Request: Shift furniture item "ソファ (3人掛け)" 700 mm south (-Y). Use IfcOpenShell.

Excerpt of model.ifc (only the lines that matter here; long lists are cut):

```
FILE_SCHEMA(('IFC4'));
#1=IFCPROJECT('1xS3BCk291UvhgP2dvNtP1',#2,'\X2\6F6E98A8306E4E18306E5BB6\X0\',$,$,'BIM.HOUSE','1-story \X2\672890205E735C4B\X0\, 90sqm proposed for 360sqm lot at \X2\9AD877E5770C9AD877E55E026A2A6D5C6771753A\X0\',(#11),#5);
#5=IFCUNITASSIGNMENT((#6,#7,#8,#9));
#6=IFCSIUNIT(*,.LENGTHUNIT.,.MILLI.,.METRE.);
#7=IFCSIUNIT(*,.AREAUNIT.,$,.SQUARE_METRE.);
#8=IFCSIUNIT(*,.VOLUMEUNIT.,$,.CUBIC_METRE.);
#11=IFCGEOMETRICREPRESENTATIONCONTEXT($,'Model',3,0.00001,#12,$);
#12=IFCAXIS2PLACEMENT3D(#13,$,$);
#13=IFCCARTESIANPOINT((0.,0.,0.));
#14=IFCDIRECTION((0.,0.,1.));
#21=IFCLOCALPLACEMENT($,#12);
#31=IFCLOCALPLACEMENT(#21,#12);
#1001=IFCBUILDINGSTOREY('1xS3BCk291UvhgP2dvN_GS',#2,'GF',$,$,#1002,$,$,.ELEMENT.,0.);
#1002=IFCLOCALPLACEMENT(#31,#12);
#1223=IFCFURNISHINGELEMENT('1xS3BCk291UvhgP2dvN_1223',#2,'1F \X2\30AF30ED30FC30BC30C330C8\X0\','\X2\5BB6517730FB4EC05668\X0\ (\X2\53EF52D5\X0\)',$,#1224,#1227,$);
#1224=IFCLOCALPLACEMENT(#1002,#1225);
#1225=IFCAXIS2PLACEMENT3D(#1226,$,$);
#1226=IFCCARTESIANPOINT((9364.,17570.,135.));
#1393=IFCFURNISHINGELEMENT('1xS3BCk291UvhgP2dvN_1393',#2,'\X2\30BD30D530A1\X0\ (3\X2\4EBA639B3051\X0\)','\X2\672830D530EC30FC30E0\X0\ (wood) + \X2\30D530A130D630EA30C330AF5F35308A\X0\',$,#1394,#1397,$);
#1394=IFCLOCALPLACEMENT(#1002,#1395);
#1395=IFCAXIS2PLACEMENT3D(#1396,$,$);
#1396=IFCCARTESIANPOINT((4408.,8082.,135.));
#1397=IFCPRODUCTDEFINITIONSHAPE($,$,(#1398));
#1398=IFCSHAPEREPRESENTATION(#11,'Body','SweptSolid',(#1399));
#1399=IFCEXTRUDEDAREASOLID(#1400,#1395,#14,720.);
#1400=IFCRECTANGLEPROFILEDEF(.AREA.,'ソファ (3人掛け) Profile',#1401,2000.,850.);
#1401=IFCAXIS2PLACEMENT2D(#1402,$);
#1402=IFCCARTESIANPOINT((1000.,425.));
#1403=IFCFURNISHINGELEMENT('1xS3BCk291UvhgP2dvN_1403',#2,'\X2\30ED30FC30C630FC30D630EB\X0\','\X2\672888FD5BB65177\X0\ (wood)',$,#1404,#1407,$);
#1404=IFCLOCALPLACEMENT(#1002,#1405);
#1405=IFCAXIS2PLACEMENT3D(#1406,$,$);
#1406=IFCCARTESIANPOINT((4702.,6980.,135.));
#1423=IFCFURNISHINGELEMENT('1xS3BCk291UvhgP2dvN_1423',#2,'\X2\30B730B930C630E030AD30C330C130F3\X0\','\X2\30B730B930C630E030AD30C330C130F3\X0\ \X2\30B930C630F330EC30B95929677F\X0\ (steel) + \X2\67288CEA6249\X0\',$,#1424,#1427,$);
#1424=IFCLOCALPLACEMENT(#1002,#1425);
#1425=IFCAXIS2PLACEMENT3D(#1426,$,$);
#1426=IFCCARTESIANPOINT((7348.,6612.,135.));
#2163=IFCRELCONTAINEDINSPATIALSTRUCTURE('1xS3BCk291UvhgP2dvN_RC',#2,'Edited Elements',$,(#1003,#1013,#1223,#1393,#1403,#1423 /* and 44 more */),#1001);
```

```python
import ifcopenshell
import ifcopenshell.api.geometry
import ifcopenshell.util.placement
import ifcopenshell.util.unit

model = ifcopenshell.open("model.ifc")
unit_scale = ifcopenshell.util.unit.calculate_unit_scale(model)

item = model.by_guid("1xS3BCk291UvhgP2dvN_1393")
matrix = ifcopenshell.util.placement.get_local_placement(item.ObjectPlacement)
matrix[1, 3] -= 0.7 / unit_scale
ifcopenshell.api.geometry.edit_object_placement(model, product=item, matrix=matrix, is_si=False)

print(ifcopenshell.util.placement.get_local_placement(item.ObjectPlacement).round(3) + 0.0)

model.write("model_rev.ifc")
```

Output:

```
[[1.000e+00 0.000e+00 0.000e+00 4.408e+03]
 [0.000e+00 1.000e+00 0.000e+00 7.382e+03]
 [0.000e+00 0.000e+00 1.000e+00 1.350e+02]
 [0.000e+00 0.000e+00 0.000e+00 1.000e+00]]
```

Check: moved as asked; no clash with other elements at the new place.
